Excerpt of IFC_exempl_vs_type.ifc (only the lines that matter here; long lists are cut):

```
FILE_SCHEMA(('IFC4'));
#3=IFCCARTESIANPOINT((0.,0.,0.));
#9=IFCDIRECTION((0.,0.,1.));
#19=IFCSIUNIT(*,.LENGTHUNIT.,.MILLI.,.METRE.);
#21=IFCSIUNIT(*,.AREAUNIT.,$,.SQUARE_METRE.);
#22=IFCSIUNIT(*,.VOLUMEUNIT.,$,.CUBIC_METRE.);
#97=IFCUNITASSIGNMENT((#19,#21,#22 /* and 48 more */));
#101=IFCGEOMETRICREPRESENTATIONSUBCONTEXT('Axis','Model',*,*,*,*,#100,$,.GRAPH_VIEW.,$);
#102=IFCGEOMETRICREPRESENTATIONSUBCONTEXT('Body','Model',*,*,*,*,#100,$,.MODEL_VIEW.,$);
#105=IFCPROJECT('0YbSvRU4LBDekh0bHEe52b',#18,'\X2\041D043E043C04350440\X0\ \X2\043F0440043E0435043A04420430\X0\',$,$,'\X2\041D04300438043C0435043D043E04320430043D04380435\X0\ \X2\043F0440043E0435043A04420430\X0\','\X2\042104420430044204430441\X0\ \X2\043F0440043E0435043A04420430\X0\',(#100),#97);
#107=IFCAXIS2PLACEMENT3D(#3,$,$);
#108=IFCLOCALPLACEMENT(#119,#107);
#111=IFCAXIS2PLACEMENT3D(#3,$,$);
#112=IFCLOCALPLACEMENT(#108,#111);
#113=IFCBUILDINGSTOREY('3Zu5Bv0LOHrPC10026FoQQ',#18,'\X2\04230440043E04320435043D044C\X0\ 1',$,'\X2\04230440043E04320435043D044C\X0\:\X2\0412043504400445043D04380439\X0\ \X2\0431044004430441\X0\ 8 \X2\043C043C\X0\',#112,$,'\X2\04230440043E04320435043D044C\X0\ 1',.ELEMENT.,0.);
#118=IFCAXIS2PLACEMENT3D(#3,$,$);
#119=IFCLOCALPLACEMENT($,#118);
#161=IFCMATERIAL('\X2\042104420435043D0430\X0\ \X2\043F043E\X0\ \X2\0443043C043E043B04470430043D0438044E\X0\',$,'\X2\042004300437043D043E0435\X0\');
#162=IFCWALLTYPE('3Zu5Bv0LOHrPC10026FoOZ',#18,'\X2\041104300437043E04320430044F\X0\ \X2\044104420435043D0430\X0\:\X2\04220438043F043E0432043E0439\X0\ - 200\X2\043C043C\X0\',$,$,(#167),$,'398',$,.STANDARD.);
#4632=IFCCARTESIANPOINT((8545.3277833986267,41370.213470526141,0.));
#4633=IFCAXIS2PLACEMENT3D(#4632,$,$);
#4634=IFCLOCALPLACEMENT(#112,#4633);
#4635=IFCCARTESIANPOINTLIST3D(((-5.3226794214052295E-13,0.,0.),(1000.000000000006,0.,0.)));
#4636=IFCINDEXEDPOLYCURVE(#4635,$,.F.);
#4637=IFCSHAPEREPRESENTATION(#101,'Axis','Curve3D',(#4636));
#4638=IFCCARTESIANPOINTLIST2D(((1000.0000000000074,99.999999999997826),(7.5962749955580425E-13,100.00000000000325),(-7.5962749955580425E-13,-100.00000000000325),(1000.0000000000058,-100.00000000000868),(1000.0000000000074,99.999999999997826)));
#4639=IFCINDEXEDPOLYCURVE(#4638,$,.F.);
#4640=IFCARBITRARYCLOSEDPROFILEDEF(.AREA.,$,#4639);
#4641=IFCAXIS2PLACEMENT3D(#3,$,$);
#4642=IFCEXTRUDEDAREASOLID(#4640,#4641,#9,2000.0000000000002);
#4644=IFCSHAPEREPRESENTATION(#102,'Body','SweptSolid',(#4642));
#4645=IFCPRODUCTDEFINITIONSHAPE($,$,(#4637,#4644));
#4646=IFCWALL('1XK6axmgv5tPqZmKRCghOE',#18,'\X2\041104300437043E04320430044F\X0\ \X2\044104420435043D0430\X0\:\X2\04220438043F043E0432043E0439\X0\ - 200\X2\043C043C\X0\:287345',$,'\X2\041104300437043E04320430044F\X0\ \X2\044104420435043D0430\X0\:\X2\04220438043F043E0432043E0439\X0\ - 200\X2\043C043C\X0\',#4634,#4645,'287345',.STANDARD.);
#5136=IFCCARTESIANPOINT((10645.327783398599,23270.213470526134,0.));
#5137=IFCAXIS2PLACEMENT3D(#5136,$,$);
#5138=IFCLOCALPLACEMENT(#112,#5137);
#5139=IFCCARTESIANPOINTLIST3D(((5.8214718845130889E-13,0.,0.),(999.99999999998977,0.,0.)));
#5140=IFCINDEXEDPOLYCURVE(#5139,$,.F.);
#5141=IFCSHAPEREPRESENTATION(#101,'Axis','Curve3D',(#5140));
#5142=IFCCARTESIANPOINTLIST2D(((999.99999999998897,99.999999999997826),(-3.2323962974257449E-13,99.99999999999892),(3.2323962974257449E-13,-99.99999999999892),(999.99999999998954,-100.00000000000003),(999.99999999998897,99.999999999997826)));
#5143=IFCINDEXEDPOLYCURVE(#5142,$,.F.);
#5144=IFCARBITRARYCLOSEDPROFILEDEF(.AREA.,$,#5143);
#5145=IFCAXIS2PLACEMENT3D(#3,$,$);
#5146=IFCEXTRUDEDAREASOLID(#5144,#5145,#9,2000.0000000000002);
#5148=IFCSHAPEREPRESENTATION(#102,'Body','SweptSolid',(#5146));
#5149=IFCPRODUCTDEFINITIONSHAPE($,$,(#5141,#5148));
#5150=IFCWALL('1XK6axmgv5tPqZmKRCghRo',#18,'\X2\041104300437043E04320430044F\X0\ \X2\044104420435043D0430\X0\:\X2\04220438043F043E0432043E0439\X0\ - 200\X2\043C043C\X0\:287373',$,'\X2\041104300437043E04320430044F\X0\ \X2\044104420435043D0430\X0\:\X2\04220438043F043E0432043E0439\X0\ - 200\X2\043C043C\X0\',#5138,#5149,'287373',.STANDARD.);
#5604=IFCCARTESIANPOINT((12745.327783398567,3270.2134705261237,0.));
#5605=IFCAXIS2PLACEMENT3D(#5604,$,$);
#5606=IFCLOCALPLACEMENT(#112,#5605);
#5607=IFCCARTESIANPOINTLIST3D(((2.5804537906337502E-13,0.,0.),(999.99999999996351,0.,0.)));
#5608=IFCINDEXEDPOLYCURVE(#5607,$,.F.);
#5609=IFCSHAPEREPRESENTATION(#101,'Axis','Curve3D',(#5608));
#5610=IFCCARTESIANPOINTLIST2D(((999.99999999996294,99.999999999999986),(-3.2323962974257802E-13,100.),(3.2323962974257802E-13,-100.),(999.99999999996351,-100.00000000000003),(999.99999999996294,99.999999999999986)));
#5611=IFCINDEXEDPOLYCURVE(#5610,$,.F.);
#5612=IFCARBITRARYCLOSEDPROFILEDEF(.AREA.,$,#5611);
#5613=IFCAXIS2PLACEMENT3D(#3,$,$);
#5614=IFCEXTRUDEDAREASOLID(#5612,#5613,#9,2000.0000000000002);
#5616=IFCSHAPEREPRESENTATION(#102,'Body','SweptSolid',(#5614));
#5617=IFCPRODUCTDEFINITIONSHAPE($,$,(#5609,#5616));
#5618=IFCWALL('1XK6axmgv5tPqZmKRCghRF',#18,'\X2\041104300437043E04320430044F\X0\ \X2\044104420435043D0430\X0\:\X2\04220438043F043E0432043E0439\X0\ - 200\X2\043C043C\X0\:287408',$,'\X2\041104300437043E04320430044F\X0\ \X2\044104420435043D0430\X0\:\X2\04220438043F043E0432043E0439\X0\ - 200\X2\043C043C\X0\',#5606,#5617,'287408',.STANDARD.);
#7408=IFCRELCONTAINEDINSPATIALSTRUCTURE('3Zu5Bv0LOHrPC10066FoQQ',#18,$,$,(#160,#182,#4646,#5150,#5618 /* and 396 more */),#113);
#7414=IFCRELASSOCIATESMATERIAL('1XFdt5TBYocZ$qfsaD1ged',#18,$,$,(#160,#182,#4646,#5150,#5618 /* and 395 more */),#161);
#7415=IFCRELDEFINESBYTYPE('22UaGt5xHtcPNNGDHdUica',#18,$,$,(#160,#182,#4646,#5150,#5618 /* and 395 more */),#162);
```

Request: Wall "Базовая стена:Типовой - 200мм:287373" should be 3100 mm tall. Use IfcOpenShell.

```python
import ifcopenshell
import ifcopenshell.geom
import ifcopenshell.util.representation
import ifcopenshell.util.shape

model = ifcopenshell.open("IFC_exempl_vs_type.ifc")
settings = ifcopenshell.geom.settings()


def volume(element):
    """Net volume in cubic metres, openings subtracted."""
    shape = ifcopenshell.geom.create_shape(settings, element)
    return ifcopenshell.util.shape.get_volume(shape.geometry)


wall = model.by_guid("1XK6axmgv5tPqZmKRCghRo")
before = volume(wall)

body = ifcopenshell.util.representation.get_representation(wall, "Model", "Body")
solid = body.Items[0]
old_height = solid.Depth
solid.Depth = 3100.0
after = volume(wall)

print(f"height {old_height:g} -> {solid.Depth:g}, volume {before:.3f} -> {after:.3f} m3")

model.write("IFC_exempl_vs_type-out.ifc")
```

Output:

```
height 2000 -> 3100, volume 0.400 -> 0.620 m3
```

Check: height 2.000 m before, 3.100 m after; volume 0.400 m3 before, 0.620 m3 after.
